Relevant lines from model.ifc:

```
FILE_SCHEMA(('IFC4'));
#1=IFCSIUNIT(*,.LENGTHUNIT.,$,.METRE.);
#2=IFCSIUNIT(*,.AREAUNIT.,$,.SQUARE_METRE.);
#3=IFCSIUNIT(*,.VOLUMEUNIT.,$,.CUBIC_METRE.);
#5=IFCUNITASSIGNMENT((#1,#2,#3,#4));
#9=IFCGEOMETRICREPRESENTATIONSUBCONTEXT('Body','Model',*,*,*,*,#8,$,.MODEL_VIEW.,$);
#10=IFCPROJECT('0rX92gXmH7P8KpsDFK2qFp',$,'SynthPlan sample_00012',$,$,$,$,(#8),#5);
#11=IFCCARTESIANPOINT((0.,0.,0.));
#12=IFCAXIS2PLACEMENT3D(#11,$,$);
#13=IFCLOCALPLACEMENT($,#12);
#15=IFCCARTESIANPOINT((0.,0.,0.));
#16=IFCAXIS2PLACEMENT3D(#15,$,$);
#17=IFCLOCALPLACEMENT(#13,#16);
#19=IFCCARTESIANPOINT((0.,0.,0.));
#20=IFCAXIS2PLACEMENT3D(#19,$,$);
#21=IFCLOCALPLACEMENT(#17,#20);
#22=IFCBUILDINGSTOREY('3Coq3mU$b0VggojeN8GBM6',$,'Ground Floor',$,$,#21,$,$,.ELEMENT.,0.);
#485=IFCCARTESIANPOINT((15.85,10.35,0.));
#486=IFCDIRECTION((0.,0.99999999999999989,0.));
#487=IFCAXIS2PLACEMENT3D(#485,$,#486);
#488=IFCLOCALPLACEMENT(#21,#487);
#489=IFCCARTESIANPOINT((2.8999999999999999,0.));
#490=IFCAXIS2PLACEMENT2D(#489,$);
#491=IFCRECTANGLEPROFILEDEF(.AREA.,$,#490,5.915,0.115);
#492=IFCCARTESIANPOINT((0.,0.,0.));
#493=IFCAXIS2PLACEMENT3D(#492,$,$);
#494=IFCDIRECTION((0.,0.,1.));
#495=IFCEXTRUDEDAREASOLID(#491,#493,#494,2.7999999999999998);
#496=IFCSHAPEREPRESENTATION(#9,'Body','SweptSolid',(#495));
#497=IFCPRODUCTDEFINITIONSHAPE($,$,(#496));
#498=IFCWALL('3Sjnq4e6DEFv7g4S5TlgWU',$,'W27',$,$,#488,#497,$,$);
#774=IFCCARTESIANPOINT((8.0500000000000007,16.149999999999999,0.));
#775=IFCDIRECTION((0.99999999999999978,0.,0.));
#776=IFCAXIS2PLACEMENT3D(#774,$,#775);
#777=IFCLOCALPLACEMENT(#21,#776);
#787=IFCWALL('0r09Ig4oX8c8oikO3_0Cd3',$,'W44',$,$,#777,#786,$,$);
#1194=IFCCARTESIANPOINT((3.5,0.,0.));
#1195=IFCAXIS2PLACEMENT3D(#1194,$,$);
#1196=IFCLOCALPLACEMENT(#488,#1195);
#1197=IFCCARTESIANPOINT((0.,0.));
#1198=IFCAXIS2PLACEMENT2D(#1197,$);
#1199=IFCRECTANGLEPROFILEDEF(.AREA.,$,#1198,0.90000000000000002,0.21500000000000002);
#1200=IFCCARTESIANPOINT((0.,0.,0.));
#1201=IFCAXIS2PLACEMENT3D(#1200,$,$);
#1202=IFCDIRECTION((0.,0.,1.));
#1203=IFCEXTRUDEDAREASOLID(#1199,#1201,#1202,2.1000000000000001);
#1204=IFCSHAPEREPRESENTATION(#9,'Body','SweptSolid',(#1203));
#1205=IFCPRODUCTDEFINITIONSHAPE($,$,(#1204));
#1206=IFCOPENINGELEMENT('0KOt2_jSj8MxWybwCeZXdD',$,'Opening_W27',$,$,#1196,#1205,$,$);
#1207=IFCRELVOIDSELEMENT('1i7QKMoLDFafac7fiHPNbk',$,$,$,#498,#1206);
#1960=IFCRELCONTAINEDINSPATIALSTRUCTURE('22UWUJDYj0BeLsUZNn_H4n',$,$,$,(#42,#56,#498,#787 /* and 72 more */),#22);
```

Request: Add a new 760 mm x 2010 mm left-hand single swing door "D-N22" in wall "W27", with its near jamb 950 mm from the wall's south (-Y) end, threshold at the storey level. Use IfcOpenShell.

```python
import numpy as np
import ifcopenshell
import ifcopenshell.api.feature
import ifcopenshell.api.geometry
import ifcopenshell.api.root
import ifcopenshell.api.spatial
import ifcopenshell.geom
import ifcopenshell.util.element
import ifcopenshell.util.placement
import ifcopenshell.util.representation
import ifcopenshell.util.shape
import ifcopenshell.util.unit

model = ifcopenshell.open("model.ifc")
unit_scale = ifcopenshell.util.unit.calculate_unit_scale(model)
settings = ifcopenshell.geom.settings()


def volume(element):
    """Net volume in cubic metres, openings subtracted."""
    shape = ifcopenshell.geom.create_shape(settings, element)
    return ifcopenshell.util.shape.get_volume(shape.geometry)


wall = model.by_guid("3Sjnq4e6DEFv7g4S5TlgWU")
storey = ifcopenshell.util.element.get_container(wall, ifc_class="IfcBuildingStorey")
context = ifcopenshell.util.representation.get_context(model, "Model", "Body", "MODEL_VIEW")
before = volume(wall)

width, height, from_end, sill = 0.76, 2.01, 0.95, 0.0  # metres

# The wall runs along its own X axis, and the end named is its -X end.
wall_shape = ifcopenshell.geom.create_shape(settings, wall)
x, y, z = ifcopenshell.util.shape.get_vertices(wall_shape.geometry).T
start = x.min() + from_end
face, thickness = float(y.min()), float(y.max() - y.min())
wall_matrix = ifcopenshell.util.placement.get_local_placement(wall.ObjectPlacement)
level = ifcopenshell.util.placement.get_local_placement(storey.ObjectPlacement)[2, 3]


def in_wall(x, y):
    """Placement at x, y metres in the wall's axes, at sill height."""
    matrix = wall_matrix.copy()
    matrix[:, 3] = wall_matrix @ np.array([x / unit_scale, y / unit_scale, 0.0, 1.0])
    matrix[2, 3] = level + sill / unit_scale
    return matrix


# Opening: a box that overshoots both wall faces by 50 mm.
opening = ifcopenshell.api.root.create_entity(model, ifc_class="IfcOpeningElement", predefined_type="OPENING")
box = ifcopenshell.api.geometry.add_wall_representation(
    model, context=context, length=width, height=height, thickness=thickness + 0.1
)
ifcopenshell.api.geometry.assign_representation(model, product=opening, representation=box)
ifcopenshell.api.geometry.edit_object_placement(model, product=opening, matrix=in_wall(start, face - 0.05), is_si=False)
ifcopenshell.api.feature.add_feature(model, feature=opening, element=wall)

door = ifcopenshell.api.root.create_entity(model, ifc_class="IfcDoor", name="D-N22", predefined_type="DOOR")
door.OverallWidth, door.OverallHeight = width / unit_scale, height / unit_scale
door.OperationType = "SINGLE_SWING_LEFT"
body = ifcopenshell.api.geometry.add_door_representation(
    model,
    context=context,
    overall_width=door.OverallWidth,
    overall_height=door.OverallHeight,
    operation_type="SINGLE_SWING_LEFT",
    lining_properties={"LiningDepth": thickness / unit_scale, "ThresholdDepth": thickness / unit_scale},
)
ifcopenshell.api.geometry.assign_representation(model, product=door, representation=body)
ifcopenshell.api.spatial.assign_container(model, products=[door], relating_structure=storey)
ifcopenshell.api.feature.add_filling(model, opening=opening, element=door)

# The lining spans the wall, so the door starts at the wall face.
ifcopenshell.api.geometry.edit_object_placement(model, product=door, matrix=in_wall(start, face), is_si=False)

after = volume(wall)

print(f"wall volume {before:.3f} -> {after:.3f} m3")

model.write("model_edited.ifc")
```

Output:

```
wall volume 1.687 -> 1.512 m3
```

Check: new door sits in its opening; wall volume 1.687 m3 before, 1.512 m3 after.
